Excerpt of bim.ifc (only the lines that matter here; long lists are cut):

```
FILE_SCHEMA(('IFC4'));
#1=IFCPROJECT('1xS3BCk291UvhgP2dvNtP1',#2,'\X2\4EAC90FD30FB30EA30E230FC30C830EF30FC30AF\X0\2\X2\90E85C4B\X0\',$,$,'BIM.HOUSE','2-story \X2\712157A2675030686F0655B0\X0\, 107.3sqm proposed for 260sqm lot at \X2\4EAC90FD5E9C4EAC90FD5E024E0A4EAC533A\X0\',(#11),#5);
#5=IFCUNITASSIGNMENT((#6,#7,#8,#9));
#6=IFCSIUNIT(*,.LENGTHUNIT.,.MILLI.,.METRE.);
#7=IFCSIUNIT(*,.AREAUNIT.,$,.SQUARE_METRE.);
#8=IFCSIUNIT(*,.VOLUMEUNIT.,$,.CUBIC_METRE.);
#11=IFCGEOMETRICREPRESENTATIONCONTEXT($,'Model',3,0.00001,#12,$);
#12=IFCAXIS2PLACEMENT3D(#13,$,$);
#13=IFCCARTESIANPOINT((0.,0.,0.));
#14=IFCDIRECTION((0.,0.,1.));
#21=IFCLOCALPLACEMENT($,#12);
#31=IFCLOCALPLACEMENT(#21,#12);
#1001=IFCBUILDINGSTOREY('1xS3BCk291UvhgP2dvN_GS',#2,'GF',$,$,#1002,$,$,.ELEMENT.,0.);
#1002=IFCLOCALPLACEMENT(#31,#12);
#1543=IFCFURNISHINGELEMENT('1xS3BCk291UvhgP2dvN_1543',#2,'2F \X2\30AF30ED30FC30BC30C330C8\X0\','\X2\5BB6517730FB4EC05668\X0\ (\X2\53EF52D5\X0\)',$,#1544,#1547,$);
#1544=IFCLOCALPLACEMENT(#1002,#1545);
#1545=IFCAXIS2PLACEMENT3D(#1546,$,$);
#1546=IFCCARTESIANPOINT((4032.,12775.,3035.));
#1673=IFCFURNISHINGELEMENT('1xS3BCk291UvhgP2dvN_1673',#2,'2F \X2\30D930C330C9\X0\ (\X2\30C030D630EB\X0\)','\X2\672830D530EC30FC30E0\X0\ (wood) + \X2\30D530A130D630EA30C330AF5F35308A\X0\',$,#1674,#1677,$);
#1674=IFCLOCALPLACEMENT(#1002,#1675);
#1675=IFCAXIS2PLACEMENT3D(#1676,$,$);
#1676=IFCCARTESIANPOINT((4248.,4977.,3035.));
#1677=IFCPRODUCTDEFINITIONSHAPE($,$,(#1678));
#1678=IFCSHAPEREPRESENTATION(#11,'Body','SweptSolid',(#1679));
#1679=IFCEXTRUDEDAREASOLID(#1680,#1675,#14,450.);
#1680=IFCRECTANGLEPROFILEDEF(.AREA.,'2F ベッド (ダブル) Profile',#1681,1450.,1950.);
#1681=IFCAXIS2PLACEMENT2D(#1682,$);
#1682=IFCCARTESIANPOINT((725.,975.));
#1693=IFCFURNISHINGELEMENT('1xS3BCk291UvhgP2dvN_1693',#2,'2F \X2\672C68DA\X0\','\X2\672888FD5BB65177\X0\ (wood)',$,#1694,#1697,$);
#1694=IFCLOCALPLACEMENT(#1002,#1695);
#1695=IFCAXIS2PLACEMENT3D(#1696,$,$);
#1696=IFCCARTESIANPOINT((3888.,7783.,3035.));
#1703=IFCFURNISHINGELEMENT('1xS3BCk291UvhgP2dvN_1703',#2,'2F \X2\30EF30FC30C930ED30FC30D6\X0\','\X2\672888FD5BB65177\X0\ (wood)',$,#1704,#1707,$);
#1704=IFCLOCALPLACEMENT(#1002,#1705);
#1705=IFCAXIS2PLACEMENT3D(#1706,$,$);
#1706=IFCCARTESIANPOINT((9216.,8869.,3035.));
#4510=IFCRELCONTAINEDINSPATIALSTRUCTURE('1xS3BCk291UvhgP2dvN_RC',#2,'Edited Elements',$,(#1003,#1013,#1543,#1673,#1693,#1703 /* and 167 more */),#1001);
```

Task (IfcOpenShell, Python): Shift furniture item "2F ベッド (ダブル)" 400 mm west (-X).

```python
import ifcopenshell
import ifcopenshell.api.geometry
import ifcopenshell.util.placement
import ifcopenshell.util.unit

model = ifcopenshell.open("bim.ifc")
unit_scale = ifcopenshell.util.unit.calculate_unit_scale(model)

item = model.by_id(1673)
matrix = ifcopenshell.util.placement.get_local_placement(item.ObjectPlacement)
matrix[0, 3] -= 0.4 / unit_scale
ifcopenshell.api.geometry.edit_object_placement(model, product=item, matrix=matrix, is_si=False)

print(ifcopenshell.util.placement.get_local_placement(item.ObjectPlacement).round(3) + 0.0)

model.write("bim_updated.ifc")
```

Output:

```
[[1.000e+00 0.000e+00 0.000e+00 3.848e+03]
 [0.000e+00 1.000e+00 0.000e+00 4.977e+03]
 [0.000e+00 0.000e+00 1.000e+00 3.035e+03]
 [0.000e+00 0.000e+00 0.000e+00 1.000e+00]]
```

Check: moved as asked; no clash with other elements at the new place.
